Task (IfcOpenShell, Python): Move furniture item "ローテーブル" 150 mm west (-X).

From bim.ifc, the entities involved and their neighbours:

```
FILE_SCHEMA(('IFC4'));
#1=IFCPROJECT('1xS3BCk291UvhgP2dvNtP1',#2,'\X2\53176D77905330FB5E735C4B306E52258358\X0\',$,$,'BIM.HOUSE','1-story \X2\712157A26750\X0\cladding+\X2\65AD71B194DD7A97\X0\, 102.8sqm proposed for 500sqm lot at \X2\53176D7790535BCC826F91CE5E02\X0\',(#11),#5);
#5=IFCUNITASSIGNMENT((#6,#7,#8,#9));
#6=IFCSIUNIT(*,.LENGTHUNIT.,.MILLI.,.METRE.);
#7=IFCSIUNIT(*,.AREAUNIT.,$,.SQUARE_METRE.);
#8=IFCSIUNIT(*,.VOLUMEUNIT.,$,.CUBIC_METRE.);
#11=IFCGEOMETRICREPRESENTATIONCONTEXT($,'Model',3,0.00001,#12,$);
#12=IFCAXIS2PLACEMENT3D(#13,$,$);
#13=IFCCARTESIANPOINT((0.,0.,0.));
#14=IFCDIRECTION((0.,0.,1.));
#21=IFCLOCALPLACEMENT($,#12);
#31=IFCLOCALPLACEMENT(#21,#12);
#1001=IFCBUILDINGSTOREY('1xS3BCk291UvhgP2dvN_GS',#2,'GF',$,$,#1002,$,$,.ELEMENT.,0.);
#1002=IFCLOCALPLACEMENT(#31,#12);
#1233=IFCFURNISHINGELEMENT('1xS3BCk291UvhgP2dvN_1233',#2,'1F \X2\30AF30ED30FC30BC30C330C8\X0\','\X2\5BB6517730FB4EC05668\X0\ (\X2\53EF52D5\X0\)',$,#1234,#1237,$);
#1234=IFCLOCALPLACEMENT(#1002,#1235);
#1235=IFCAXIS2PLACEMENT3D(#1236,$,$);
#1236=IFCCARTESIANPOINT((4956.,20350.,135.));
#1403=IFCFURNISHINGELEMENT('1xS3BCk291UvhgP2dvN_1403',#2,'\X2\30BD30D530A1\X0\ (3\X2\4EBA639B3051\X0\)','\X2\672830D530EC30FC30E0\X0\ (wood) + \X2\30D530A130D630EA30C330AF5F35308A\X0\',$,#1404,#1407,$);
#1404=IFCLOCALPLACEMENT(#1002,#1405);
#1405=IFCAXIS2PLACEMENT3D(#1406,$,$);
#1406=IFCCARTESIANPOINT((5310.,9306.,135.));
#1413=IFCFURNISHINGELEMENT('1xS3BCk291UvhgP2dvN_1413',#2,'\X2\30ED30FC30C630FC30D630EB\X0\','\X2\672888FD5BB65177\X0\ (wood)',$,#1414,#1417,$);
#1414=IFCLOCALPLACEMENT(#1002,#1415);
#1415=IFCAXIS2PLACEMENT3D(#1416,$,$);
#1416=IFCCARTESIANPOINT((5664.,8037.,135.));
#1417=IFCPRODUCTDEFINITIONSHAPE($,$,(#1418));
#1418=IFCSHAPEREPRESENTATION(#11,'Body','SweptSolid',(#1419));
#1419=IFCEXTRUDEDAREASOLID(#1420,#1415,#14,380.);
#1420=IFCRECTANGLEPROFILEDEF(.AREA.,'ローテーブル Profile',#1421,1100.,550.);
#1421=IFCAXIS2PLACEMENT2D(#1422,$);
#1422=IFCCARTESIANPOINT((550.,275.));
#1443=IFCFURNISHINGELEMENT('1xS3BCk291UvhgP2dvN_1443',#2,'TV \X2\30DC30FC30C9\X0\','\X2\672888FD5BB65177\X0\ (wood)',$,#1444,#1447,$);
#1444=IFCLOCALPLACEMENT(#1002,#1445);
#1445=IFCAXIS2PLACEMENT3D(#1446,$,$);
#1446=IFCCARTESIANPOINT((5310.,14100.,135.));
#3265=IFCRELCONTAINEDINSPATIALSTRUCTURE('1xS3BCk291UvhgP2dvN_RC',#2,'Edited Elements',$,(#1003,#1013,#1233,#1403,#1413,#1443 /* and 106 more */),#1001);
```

```python
import ifcopenshell
import ifcopenshell.api.geometry
import ifcopenshell.util.placement
import ifcopenshell.util.unit

model = ifcopenshell.open("bim.ifc")
unit_scale = ifcopenshell.util.unit.calculate_unit_scale(model)

item = model.by_guid("1xS3BCk291UvhgP2dvN_1413")
matrix = ifcopenshell.util.placement.get_local_placement(item.ObjectPlacement)
matrix[0, 3] -= 0.15 / unit_scale
ifcopenshell.api.geometry.edit_object_placement(model, product=item, matrix=matrix, is_si=False)

print(ifcopenshell.util.placement.get_local_placement(item.ObjectPlacement).round(3) + 0.0)

model.write("bim-out.ifc")
```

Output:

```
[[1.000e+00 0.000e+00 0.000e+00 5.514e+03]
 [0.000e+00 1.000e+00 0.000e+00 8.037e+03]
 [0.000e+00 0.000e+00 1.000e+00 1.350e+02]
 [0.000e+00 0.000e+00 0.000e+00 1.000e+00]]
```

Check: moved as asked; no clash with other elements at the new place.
